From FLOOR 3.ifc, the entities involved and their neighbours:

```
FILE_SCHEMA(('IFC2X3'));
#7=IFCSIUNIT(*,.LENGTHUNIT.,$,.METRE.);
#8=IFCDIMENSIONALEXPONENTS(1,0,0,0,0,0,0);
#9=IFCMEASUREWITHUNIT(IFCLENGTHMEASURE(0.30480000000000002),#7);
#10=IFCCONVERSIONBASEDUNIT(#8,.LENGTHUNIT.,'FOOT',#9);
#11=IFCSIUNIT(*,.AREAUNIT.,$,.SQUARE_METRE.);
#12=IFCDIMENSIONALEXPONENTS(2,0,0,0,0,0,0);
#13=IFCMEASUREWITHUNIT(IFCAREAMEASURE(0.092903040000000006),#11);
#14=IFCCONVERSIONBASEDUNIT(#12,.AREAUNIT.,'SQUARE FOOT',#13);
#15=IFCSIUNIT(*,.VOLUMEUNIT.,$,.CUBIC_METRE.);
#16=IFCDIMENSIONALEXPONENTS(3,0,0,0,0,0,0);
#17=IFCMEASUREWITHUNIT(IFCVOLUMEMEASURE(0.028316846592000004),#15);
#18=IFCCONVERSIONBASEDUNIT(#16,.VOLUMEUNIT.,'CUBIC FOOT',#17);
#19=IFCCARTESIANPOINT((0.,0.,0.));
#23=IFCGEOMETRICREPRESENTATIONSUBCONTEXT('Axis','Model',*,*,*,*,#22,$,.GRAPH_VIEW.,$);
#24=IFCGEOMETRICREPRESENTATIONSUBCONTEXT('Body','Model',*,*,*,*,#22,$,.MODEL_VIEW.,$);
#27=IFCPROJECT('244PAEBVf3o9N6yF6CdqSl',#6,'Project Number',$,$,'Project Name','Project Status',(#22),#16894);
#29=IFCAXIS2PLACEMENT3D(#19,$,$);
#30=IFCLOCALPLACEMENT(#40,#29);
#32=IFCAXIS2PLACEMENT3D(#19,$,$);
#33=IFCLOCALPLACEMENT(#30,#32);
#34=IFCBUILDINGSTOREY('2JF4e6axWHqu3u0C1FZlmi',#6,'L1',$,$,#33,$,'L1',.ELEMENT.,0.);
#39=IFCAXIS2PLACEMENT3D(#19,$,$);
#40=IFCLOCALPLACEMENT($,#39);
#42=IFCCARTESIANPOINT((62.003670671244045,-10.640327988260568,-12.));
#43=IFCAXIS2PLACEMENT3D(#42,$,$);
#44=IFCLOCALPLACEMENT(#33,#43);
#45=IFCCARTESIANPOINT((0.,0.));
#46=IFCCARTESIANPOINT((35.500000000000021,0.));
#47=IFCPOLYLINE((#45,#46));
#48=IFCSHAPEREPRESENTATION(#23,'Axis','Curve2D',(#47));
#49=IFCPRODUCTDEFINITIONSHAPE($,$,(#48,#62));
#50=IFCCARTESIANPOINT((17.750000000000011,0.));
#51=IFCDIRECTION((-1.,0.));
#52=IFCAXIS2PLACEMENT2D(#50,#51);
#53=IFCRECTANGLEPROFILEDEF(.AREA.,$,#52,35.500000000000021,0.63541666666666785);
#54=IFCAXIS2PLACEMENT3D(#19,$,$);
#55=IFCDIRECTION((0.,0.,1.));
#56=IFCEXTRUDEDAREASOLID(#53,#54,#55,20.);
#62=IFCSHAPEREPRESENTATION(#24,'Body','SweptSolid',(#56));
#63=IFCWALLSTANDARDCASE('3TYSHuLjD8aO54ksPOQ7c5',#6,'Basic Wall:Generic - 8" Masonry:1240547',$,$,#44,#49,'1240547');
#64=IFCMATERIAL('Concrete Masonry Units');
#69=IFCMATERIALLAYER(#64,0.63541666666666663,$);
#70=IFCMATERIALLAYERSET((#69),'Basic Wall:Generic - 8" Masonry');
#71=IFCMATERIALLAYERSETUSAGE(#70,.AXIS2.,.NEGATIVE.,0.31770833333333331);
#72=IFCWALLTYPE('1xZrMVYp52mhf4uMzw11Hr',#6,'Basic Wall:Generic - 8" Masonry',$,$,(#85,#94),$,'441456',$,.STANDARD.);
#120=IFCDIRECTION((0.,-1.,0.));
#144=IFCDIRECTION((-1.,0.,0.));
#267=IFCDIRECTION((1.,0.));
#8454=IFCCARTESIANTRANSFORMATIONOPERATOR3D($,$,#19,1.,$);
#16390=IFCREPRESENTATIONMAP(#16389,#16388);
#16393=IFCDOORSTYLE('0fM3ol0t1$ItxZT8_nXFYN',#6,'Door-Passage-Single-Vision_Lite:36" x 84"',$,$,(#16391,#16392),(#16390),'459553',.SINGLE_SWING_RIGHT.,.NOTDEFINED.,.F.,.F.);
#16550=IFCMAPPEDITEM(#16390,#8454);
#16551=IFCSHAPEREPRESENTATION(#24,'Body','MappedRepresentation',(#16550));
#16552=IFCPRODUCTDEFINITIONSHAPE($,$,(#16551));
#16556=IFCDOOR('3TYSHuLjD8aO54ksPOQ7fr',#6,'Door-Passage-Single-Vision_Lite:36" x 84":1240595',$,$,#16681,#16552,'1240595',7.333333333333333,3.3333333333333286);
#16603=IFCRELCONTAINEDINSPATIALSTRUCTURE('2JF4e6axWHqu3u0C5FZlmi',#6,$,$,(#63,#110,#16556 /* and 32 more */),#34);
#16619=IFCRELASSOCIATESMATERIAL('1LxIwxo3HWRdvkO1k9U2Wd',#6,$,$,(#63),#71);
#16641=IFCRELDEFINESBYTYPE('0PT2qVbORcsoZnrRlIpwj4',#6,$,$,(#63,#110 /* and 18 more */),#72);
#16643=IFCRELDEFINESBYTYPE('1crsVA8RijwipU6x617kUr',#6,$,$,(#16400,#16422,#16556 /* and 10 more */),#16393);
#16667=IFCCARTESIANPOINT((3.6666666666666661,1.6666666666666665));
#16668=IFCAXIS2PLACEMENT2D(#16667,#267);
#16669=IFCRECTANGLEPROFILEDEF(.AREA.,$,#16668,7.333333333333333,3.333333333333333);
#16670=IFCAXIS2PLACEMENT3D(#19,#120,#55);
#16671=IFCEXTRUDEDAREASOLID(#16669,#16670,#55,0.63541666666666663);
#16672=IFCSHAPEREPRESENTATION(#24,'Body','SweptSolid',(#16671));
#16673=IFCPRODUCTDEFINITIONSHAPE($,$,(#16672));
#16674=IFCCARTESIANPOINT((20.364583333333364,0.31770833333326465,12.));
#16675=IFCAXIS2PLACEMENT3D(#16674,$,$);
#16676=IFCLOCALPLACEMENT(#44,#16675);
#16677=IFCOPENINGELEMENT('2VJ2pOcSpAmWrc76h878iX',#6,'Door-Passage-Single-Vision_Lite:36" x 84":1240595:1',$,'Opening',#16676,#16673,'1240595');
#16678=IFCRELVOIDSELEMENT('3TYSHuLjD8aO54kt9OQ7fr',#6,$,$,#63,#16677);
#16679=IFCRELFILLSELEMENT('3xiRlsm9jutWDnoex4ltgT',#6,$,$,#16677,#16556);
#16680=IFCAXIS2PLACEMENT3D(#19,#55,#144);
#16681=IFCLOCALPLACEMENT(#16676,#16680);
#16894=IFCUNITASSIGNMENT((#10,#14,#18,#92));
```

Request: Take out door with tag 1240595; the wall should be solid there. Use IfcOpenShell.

```python
import ifcopenshell
import ifcopenshell.api.feature
import ifcopenshell.api.root
import ifcopenshell.geom
import ifcopenshell.util.shape

model = ifcopenshell.open("FLOOR 3.ifc")
settings = ifcopenshell.geom.settings()


def volume(element):
    """Net volume in cubic metres, openings subtracted."""
    shape = ifcopenshell.geom.create_shape(settings, element)
    return ifcopenshell.util.shape.get_volume(shape.geometry)


door = model.by_guid("3TYSHuLjD8aO54ksPOQ7fr")
opening = door.FillsVoids[0].RelatingOpeningElement
wall = opening.VoidsElements[0].RelatingBuildingElement
before = volume(wall)

ifcopenshell.api.root.remove_product(model, product=door)
ifcopenshell.api.feature.remove_feature(model, feature=opening)

after = volume(wall)

print(f"wall volume {before:.3f} -> {after:.3f} m3")

model.write("FLOOR 3_rev.ifc")
```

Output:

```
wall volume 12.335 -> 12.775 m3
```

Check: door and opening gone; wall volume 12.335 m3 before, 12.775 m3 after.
